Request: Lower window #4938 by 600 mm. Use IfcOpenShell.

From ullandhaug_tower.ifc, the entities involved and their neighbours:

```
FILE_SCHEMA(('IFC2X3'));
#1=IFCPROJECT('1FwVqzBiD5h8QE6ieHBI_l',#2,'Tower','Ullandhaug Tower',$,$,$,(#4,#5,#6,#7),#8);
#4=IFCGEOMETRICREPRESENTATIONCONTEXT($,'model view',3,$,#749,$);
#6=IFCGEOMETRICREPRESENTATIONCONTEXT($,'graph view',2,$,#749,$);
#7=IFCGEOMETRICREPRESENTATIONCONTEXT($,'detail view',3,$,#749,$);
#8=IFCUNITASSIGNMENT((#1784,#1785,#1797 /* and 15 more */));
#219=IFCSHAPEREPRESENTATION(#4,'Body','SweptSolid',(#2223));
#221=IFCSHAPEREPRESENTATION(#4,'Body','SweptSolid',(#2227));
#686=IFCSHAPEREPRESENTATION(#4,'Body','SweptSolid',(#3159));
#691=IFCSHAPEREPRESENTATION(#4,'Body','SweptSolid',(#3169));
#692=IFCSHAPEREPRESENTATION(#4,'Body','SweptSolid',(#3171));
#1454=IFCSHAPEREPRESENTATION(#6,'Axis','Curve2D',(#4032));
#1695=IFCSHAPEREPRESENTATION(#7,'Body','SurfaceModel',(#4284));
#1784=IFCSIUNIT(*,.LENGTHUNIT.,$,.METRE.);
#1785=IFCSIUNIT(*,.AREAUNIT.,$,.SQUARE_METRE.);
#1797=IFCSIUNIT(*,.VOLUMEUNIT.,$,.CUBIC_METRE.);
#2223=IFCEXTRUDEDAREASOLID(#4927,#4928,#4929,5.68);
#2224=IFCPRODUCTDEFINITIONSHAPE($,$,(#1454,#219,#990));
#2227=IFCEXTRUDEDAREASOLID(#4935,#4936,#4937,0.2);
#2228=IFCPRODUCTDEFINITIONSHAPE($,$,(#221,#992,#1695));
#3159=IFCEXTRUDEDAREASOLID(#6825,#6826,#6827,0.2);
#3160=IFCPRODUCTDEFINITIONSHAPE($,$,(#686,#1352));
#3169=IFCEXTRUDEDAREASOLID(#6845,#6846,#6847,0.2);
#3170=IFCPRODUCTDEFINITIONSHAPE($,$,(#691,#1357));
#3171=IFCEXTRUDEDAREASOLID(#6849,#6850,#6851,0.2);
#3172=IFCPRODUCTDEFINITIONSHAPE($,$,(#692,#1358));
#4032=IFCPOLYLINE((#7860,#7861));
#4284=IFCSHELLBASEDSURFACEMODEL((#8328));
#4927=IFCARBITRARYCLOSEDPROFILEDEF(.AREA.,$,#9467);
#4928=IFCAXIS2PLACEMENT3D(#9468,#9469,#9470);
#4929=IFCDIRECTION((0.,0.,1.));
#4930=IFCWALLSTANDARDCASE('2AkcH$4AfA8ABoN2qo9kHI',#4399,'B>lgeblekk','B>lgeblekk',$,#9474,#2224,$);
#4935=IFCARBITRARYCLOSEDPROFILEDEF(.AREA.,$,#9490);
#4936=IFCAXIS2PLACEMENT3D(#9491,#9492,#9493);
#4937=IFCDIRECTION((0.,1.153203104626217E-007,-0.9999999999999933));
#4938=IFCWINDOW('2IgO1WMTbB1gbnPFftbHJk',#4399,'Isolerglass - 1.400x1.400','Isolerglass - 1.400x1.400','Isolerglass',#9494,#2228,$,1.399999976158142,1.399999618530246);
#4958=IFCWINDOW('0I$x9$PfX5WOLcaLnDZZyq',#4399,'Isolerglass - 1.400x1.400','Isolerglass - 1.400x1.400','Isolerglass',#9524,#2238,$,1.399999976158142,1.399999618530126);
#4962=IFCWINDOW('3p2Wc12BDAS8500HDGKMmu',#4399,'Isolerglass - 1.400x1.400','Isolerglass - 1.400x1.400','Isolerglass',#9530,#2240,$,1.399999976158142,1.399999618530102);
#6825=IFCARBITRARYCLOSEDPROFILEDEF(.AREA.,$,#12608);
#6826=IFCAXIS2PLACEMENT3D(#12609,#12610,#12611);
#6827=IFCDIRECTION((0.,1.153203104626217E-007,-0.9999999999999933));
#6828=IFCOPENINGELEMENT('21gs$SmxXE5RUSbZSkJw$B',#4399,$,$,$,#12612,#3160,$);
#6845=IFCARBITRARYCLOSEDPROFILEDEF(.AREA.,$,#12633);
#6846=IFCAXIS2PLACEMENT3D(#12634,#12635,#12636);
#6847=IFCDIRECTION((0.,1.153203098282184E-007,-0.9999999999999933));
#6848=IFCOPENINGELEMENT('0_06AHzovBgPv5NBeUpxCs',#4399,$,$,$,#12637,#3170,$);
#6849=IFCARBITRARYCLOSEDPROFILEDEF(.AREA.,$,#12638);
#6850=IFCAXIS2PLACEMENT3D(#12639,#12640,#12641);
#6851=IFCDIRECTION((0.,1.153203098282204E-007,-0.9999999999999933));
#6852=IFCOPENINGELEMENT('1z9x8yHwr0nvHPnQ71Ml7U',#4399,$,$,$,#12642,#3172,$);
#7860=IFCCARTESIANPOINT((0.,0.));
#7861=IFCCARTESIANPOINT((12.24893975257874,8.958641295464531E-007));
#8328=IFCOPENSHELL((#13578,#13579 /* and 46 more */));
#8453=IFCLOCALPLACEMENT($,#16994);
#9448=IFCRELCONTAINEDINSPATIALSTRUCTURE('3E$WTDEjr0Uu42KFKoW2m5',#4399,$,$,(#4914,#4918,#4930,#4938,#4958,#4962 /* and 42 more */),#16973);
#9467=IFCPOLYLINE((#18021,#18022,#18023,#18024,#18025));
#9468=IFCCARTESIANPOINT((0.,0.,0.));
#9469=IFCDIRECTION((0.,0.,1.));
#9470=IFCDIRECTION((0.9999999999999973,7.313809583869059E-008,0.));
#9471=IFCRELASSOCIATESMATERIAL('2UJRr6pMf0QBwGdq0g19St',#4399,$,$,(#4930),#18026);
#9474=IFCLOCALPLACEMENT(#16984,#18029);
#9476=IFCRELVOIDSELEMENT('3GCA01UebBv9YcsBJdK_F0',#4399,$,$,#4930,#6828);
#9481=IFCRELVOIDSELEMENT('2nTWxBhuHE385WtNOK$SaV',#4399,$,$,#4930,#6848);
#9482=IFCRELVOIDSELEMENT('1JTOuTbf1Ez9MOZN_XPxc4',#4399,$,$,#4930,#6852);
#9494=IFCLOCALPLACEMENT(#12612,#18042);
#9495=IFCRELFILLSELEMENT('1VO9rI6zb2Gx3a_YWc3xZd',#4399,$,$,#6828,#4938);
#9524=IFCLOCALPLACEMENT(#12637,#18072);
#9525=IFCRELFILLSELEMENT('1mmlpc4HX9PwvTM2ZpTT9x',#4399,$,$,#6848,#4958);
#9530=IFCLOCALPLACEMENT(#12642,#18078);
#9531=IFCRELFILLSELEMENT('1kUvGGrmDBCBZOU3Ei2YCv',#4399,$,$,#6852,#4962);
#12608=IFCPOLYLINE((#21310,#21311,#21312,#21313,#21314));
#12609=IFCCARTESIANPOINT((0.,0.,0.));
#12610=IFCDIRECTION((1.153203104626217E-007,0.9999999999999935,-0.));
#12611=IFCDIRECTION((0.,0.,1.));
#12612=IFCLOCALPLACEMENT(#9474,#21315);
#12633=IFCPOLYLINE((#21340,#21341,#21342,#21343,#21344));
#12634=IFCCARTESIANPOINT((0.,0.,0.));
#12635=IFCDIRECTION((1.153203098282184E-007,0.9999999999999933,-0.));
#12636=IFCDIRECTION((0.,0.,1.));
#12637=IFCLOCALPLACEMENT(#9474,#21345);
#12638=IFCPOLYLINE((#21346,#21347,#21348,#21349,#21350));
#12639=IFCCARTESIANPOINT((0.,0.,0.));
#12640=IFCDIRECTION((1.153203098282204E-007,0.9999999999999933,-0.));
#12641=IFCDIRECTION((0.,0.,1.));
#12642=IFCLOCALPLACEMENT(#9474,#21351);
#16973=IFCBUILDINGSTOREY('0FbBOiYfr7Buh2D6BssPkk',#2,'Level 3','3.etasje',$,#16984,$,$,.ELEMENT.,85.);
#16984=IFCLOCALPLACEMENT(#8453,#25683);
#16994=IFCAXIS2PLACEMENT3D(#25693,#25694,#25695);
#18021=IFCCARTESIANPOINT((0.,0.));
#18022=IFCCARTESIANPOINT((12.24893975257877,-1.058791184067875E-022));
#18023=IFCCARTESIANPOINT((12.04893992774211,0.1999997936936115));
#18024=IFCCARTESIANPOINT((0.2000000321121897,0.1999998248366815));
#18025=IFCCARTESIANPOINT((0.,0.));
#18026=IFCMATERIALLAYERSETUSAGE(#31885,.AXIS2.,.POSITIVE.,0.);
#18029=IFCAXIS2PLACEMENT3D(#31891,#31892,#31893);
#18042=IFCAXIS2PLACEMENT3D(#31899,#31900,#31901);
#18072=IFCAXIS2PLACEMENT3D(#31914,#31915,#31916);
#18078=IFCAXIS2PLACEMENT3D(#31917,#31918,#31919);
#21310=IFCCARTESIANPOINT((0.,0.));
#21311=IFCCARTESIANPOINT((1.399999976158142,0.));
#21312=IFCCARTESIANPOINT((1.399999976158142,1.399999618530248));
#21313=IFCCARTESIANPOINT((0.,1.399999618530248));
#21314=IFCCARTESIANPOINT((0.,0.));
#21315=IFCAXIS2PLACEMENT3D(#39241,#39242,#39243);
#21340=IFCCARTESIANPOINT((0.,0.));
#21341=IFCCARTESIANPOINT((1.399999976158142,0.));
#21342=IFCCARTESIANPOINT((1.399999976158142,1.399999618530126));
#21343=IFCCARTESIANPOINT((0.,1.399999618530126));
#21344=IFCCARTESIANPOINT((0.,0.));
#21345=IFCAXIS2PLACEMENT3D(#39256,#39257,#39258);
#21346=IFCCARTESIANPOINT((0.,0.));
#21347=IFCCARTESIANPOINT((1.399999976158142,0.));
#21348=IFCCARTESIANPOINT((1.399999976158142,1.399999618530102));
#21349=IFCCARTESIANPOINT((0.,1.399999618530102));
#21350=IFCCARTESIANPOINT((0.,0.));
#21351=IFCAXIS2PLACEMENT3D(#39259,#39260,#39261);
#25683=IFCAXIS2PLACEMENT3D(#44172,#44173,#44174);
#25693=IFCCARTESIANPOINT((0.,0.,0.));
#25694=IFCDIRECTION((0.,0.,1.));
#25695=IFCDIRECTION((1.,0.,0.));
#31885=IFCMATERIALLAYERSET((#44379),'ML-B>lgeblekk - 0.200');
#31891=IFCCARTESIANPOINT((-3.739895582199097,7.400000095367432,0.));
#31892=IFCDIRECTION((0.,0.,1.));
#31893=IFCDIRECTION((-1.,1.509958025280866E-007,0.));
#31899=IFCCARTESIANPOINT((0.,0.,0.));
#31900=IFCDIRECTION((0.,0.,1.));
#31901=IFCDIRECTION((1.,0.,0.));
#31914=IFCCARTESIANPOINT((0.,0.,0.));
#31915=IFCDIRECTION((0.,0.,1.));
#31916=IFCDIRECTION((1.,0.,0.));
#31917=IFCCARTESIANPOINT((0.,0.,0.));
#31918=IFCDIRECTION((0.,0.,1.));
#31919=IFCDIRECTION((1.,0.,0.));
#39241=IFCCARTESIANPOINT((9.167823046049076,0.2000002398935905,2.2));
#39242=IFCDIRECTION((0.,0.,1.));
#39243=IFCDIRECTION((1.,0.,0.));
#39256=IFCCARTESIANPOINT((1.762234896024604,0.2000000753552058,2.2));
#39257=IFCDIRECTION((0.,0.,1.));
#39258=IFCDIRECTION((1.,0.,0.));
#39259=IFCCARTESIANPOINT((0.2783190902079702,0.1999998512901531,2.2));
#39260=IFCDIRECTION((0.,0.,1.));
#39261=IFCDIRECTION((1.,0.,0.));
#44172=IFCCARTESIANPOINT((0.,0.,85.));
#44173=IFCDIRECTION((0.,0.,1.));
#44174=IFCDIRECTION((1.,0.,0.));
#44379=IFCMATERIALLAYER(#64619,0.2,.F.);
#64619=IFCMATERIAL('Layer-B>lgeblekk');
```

```python
import numpy as np
import ifcopenshell
import ifcopenshell.api.geometry
import ifcopenshell.util.placement
import ifcopenshell.util.unit

model = ifcopenshell.open("ullandhaug_tower.ifc")
unit_scale = ifcopenshell.util.unit.calculate_unit_scale(model)

window = model.by_guid("2IgO1WMTbB1gbnPFftbHJk")
opening = window.FillsVoids[0].RelatingOpeningElement
dz = -0.6 / unit_scale

shift = np.array([0.0, 0.0, dz])
# The window is placed relative to its opening, so it follows when the opening moves.
matrix = ifcopenshell.util.placement.get_local_placement(opening.ObjectPlacement)
matrix[:3, 3] += shift
ifcopenshell.api.geometry.edit_object_placement(
    model, product=opening, matrix=matrix, is_si=False, should_transform_children=True
)

print(f"moved by {dz * unit_scale:+.3f} m")

model.write("ullandhaug_tower_updated.ifc")
```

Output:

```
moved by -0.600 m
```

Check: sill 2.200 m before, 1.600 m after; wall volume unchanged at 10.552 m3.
